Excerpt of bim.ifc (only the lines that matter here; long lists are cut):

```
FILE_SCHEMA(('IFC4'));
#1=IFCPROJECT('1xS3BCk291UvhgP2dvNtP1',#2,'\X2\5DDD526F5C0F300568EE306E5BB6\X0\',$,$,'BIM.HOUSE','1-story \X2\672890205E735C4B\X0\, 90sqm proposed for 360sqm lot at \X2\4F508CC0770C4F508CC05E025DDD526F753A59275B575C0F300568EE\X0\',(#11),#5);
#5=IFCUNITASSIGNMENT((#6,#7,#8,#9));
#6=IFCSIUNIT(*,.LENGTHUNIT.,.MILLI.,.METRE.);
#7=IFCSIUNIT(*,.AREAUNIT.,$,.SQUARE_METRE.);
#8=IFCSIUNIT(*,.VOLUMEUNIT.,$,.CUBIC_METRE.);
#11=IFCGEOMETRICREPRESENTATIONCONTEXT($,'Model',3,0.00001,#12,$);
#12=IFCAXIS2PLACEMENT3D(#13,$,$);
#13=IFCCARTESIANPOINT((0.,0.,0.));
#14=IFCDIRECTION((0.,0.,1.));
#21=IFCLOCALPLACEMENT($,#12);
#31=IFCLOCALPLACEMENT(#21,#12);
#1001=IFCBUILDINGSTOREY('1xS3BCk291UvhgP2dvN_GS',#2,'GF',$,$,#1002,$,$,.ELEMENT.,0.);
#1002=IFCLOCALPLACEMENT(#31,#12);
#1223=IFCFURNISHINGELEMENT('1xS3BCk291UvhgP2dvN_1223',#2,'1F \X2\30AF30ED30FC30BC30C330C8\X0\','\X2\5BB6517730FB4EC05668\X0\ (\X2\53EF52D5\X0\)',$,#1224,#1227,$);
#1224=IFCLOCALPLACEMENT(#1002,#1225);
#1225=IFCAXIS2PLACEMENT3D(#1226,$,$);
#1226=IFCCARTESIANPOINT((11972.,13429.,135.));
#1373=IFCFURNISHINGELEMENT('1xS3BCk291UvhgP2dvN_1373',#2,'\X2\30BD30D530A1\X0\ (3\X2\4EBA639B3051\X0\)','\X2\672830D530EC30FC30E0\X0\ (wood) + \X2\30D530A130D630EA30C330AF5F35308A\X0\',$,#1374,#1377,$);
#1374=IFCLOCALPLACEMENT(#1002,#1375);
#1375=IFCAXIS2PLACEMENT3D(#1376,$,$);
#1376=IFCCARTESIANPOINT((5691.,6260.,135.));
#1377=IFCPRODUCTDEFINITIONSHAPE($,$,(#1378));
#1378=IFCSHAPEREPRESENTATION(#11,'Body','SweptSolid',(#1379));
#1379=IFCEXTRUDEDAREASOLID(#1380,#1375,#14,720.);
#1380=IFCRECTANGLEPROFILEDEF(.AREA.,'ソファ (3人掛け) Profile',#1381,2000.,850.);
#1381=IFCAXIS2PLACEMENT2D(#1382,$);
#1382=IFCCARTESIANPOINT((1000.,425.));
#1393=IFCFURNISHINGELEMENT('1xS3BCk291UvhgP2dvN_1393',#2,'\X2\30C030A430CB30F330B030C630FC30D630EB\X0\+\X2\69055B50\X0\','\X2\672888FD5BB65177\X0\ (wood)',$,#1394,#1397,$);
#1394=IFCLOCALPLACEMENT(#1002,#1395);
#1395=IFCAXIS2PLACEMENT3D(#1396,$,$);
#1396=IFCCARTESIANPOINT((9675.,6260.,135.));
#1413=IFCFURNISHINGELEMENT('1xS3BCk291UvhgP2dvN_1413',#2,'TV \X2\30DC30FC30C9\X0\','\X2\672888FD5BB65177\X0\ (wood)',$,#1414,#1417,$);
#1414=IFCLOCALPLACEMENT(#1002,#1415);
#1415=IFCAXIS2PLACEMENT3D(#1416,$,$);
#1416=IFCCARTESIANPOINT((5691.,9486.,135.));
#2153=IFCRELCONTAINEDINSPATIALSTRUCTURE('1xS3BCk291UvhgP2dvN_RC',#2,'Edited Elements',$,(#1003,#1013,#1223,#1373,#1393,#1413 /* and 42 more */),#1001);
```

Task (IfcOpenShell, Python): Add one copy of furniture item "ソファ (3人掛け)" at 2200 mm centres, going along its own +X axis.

```python
import ifcopenshell
import ifcopenshell.api.geometry
import ifcopenshell.api.root
import ifcopenshell.util.element
import ifcopenshell.util.placement

model = ifcopenshell.open("bim.ifc")


def reuse_history(source, copy):
    """copy_class also copies each property set's owner history, people and application; keep the originals."""
    for rel in copy.IsDefinedBy:
        if rel.is_a("IfcRelDefinesByProperties") and (history := rel.RelatingPropertyDefinition.OwnerHistory):
            rel.RelatingPropertyDefinition.OwnerHistory = source.OwnerHistory
            ifcopenshell.util.element.remove_deep2(model, history)


source = model.by_id(1373)
base = ifcopenshell.util.placement.get_local_placement(source.ObjectPlacement)
step = base[:3, 0] * 2200.0

for i in range(1, 2):
    copy = ifcopenshell.api.root.copy_class(model, product=source)
    copy.Representation = ifcopenshell.util.element.copy_deep(
        model, source.Representation, exclude=["IfcGeometricRepresentationContext", "IfcRepresentationMap"]
    )
    reuse_history(source, copy)
    matrix = base.copy()
    matrix[:3, 3] += i * step
    print("added at", matrix[:3, 3].round(3) + 0.0)
    ifcopenshell.api.geometry.edit_object_placement(model, product=copy, matrix=matrix, is_si=False)

model.write("bim_edited.ifc")
```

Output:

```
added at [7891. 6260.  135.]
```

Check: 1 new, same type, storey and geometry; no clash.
